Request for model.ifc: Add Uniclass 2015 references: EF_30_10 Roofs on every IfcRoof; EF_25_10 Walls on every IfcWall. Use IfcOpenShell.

First a look at what the model holds.

```python
import ifcopenshell

model = ifcopenshell.open("model.ifc")
print(model.schema)
print("classifications:", [c.Name for c in model.by_type("IfcClassification")])
for ifc_class in ("IfcDoor", "IfcRoof", "IfcStair", "IfcWall", "IfcWindow"):
    print(ifc_class, len(model.by_type(ifc_class)))
```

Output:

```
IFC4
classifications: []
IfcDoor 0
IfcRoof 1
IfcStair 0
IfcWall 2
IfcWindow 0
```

```python
import ifcopenshell
import ifcopenshell.api.classification

model = ifcopenshell.open("model.ifc")

system = ifcopenshell.api.classification.add_classification(model, classification="Uniclass 2015")

codes = {
    "IfcRoof": ("EF_30_10", "Roofs"),
    "IfcWall": ("EF_25_10", "Walls"),
}
for ifc_class, (code, name) in codes.items():
    products = model.by_type(ifc_class)
    ifcopenshell.api.classification.add_reference(
        model, products=products, classification=system, identification=code, name=name
    )
    print(code, len(products))

model.write("model_updated.ifc")
```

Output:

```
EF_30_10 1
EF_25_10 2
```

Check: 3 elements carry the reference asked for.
